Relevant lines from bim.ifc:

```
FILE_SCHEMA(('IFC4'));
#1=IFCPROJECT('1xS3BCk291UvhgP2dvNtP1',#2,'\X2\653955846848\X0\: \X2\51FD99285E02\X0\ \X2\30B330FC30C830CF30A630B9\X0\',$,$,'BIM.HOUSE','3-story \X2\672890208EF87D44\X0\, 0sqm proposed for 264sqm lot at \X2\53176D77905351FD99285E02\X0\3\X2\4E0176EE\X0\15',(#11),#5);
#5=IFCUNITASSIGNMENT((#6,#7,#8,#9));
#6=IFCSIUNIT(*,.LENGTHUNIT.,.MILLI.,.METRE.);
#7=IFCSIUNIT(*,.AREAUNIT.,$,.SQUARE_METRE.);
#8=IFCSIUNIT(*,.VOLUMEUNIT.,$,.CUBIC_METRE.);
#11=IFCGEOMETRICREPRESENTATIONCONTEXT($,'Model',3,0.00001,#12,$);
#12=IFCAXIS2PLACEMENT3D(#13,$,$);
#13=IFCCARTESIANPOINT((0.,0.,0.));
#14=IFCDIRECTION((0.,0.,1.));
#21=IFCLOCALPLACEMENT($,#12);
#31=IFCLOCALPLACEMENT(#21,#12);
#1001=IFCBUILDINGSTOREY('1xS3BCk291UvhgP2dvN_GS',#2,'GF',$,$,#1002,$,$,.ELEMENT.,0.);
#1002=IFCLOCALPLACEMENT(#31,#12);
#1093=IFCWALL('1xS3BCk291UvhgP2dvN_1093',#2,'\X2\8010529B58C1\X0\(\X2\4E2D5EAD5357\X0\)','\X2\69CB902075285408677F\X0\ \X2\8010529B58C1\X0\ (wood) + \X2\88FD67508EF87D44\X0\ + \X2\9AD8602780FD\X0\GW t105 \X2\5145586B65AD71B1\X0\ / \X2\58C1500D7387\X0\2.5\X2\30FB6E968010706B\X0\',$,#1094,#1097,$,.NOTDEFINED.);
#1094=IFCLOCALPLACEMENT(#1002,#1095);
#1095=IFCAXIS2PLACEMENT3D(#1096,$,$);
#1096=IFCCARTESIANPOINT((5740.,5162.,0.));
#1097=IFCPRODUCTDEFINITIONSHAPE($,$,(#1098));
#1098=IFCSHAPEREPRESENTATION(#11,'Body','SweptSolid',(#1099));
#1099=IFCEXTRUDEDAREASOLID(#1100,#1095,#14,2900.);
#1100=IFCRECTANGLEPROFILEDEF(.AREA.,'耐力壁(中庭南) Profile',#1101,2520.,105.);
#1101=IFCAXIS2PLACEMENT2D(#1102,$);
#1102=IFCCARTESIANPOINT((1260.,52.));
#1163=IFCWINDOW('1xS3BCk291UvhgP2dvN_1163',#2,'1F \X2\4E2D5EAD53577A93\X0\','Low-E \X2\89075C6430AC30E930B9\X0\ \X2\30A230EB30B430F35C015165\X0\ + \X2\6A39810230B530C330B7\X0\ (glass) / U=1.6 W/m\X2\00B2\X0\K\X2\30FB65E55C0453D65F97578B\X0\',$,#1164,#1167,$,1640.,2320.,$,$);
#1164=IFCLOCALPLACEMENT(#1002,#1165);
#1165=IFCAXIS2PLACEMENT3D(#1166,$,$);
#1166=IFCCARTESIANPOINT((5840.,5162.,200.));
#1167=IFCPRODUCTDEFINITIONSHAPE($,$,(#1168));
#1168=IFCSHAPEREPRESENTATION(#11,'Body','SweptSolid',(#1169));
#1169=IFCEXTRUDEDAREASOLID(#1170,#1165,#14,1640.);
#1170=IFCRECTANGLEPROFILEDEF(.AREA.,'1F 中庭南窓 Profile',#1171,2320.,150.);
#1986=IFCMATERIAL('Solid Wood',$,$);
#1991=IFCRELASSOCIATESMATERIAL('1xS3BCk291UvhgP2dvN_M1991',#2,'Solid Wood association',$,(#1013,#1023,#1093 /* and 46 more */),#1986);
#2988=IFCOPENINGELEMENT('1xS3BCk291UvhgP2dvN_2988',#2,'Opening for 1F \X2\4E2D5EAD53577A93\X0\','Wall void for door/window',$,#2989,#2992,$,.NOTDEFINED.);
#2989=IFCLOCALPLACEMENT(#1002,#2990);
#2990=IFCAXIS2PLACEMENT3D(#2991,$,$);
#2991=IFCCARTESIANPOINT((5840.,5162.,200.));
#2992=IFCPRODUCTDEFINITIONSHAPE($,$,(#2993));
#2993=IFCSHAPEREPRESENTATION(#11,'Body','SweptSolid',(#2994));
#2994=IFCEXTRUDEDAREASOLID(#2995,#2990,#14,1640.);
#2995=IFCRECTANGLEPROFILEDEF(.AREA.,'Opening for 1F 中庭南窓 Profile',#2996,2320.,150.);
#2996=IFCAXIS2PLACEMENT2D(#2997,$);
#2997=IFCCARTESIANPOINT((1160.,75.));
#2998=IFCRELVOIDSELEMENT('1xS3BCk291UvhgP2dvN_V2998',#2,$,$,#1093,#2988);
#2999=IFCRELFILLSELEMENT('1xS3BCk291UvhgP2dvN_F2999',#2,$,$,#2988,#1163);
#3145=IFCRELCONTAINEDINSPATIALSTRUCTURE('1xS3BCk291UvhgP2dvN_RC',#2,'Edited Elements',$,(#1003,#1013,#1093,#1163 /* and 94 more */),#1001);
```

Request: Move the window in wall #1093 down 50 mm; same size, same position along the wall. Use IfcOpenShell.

```python
import numpy as np
import ifcopenshell
import ifcopenshell.api.geometry
import ifcopenshell.util.placement
import ifcopenshell.util.unit

model = ifcopenshell.open("bim.ifc")
unit_scale = ifcopenshell.util.unit.calculate_unit_scale(model)

window = model.by_guid("1xS3BCk291UvhgP2dvN_1163")
opening = window.FillsVoids[0].RelatingOpeningElement
dz = -0.05 / unit_scale

shift = np.array([0.0, 0.0, dz])
# The window is not placed relative to its opening, so move both.
for product in (opening, window):
    matrix = ifcopenshell.util.placement.get_local_placement(product.ObjectPlacement)
    matrix[:3, 3] += shift
    ifcopenshell.api.geometry.edit_object_placement(model, product=product, matrix=matrix, is_si=False)

print(f"moved by {dz * unit_scale:+.3f} m")

model.write("bim_updated.ifc")
```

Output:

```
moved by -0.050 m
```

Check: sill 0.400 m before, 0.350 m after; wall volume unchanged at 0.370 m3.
